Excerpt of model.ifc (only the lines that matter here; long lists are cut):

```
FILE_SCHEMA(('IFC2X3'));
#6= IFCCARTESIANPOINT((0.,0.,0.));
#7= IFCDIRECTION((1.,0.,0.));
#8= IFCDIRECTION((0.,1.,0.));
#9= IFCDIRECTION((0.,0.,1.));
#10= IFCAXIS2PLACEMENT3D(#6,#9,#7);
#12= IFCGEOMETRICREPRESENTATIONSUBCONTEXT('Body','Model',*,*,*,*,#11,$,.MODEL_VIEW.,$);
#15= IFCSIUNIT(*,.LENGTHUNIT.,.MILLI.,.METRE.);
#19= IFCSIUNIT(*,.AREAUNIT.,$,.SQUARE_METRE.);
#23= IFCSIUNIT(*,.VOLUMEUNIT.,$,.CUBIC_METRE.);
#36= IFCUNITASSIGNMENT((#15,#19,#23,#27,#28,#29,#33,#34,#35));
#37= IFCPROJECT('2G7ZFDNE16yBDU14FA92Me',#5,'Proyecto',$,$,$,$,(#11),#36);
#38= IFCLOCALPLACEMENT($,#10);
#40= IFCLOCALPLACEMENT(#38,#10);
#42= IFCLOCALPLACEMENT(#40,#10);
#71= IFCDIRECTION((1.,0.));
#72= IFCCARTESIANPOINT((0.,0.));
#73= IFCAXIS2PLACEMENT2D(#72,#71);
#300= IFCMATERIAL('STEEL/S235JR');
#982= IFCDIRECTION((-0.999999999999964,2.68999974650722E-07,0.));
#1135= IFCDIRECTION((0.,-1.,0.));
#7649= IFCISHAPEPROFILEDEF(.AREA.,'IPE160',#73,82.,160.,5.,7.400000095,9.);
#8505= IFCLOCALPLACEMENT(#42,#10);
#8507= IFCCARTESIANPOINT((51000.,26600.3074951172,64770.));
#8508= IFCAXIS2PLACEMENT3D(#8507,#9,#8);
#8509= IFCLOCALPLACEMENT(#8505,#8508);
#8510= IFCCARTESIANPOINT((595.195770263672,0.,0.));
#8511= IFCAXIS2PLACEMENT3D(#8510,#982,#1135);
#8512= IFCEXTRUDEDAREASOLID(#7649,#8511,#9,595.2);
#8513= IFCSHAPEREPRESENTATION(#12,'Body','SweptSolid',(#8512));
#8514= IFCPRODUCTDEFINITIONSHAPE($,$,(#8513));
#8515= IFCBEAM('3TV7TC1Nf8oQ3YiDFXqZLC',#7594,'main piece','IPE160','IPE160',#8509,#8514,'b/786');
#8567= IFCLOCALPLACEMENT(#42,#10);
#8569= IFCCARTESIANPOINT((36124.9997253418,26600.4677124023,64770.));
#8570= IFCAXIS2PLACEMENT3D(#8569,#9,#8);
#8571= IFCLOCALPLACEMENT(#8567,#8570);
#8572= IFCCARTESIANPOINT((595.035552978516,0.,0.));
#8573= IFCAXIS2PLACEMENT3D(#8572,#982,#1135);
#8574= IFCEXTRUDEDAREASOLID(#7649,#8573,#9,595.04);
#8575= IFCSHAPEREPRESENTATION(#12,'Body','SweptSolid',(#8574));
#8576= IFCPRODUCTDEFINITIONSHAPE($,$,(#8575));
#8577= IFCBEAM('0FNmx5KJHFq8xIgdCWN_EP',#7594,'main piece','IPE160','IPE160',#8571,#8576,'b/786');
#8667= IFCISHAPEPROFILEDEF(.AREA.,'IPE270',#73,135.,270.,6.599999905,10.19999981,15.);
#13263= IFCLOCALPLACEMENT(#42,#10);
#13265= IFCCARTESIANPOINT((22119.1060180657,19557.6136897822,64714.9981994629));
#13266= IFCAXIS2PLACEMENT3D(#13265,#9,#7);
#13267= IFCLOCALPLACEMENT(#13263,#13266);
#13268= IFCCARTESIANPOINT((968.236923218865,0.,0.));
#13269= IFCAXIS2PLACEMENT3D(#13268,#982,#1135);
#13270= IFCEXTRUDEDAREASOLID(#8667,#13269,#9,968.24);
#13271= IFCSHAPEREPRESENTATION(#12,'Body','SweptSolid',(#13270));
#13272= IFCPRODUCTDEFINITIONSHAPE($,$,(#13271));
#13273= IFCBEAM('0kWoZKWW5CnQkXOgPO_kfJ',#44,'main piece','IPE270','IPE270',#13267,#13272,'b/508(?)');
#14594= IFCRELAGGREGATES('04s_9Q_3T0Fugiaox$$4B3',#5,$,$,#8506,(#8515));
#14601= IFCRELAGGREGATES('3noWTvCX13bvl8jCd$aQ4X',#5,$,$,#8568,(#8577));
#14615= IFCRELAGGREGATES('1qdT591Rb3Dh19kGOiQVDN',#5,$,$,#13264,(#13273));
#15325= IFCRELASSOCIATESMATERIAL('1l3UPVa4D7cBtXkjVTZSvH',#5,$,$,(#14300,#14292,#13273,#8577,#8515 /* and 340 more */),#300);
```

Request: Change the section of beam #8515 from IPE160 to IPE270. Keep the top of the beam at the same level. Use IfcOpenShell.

```python
import ifcopenshell
import ifcopenshell.util.element
import ifcopenshell.util.representation

model = ifcopenshell.open("model.ifc")

member = model.by_guid("3TV7TC1Nf8oQ3YiDFXqZLC")
source = next(p for p in model.by_type("IfcIShapeProfileDef") if p.ProfileName == "IPE270")

body = ifcopenshell.util.representation.get_representation(member, "Model", "Body")
solid = body.Items[0]
old_profile = solid.SweptArea

# Copy the section's sizes but keep this member's own profile position.
profile = ifcopenshell.util.element.copy(model, source)
# Profiles are centred, so shift by half the change in depth to hold the top.
shift = (old_profile.OverallDepth - profile.OverallDepth) / 2
x, y = old_profile.Position.Location.Coordinates
up = (0.0, 1.0)  # upwards, in the solid's own plane
location = model.createIfcCartesianPoint((x + up[0] * shift, y + up[1] * shift))
profile.Position = model.createIfcAxis2Placement2D(location, old_profile.Position.RefDirection)
solid.SweptArea = profile
if not model.get_total_inverses(old_profile):
    ifcopenshell.util.element.remove_deep2(model, old_profile)
member.Description = member.Description.replace("IPE160", "IPE270")
member.ObjectType = member.ObjectType.replace("IPE160", "IPE270")

print(solid.SweptArea)

model.write("model_edited.ifc")
```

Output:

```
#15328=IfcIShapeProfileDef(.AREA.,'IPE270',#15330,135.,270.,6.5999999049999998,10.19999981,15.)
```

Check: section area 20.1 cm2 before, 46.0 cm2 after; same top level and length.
